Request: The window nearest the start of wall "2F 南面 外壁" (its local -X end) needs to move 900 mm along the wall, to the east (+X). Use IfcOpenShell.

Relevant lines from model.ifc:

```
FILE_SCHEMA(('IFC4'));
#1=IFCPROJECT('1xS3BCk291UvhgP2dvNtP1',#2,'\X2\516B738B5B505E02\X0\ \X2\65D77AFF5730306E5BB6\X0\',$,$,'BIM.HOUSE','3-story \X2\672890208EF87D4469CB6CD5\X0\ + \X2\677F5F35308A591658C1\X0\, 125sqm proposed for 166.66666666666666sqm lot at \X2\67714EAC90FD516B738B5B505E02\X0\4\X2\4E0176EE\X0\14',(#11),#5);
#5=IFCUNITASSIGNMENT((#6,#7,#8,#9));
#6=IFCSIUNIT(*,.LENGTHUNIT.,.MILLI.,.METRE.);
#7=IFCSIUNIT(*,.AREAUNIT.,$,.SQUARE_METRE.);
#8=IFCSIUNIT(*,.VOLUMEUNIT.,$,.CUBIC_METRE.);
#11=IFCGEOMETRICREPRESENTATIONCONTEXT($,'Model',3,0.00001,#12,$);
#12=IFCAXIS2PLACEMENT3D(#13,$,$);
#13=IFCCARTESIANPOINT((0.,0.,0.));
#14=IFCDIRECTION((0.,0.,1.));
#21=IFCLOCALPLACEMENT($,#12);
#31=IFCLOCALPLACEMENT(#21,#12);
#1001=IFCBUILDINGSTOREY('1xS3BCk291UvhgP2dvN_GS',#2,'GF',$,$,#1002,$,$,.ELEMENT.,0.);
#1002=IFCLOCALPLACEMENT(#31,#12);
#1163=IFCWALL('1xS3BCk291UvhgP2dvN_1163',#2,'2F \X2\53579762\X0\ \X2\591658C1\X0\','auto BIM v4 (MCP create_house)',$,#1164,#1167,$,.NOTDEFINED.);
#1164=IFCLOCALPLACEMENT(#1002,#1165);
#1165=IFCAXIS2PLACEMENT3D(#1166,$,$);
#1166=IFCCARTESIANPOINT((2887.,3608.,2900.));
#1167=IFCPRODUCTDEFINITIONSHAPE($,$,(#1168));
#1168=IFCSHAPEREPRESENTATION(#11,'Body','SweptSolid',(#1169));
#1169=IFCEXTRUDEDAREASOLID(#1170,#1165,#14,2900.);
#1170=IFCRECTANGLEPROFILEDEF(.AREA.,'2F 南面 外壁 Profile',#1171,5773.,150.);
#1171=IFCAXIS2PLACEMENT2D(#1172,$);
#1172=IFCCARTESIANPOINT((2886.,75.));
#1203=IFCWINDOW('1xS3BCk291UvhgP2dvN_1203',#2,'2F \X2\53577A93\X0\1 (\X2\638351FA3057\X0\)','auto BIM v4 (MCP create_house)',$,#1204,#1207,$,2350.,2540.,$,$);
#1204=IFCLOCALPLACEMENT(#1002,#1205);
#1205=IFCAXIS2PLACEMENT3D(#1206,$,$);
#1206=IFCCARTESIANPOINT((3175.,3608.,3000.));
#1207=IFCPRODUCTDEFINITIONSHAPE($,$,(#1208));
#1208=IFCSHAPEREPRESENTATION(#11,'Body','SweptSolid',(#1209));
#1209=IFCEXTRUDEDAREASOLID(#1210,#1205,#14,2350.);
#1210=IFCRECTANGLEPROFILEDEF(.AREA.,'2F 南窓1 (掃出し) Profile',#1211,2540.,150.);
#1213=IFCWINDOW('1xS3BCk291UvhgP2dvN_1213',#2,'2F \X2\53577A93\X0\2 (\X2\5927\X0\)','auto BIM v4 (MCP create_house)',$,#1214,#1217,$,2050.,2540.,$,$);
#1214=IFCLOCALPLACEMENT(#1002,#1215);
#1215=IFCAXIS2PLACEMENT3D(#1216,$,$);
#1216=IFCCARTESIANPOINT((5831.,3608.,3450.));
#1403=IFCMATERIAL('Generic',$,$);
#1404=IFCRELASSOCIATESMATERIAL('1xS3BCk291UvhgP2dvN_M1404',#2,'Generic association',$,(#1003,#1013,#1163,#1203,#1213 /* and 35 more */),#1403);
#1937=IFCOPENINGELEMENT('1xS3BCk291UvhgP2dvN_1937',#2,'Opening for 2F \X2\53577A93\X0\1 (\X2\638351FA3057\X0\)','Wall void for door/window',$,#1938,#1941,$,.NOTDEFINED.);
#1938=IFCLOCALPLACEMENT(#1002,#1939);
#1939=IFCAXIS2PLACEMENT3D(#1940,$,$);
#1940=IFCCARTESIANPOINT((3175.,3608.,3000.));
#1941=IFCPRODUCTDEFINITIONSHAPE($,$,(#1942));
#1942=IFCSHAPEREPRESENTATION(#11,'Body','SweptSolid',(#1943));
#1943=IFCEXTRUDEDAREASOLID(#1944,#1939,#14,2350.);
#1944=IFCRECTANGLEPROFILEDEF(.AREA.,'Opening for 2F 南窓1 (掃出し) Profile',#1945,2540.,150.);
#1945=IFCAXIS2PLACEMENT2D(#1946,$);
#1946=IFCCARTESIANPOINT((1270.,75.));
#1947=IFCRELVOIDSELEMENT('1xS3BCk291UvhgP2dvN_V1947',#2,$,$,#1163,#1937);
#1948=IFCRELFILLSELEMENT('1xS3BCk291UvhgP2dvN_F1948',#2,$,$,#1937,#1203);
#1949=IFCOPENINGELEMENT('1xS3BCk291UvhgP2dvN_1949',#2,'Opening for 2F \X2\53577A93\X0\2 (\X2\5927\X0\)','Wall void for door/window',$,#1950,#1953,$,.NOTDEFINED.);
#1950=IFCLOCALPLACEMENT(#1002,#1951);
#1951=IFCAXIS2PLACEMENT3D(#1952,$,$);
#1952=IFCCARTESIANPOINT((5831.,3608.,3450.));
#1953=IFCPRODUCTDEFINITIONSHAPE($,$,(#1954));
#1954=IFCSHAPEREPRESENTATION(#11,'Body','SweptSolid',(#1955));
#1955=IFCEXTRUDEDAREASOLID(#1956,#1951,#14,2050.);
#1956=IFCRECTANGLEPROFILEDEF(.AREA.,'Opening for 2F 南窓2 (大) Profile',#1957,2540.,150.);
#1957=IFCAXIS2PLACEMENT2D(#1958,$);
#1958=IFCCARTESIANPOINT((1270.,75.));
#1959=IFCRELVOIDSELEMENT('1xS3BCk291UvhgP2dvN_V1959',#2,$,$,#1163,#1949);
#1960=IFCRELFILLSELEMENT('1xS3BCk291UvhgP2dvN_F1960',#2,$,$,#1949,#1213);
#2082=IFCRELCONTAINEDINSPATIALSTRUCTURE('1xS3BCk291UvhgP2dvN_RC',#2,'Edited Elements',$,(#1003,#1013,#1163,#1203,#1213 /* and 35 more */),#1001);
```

```python
import ifcopenshell
import ifcopenshell.api.geometry
import ifcopenshell.util.placement

model = ifcopenshell.open("model.ifc")

window = model.by_guid("1xS3BCk291UvhgP2dvN_1203")
opening = window.FillsVoids[0].RelatingOpeningElement
wall = opening.VoidsElements[0].RelatingBuildingElement

wall_matrix = ifcopenshell.util.placement.get_local_placement(wall.ObjectPlacement)
shift = wall_matrix[:3, 0] * 900.0
before = ifcopenshell.util.placement.get_local_placement(window.ObjectPlacement)[:3, 3].copy()

# The window is not placed relative to its opening, so move both.
for product in (opening, window):
    matrix = ifcopenshell.util.placement.get_local_placement(product.ObjectPlacement)
    matrix[:3, 3] += shift
    ifcopenshell.api.geometry.edit_object_placement(model, product=product, matrix=matrix, is_si=False)

after = ifcopenshell.util.placement.get_local_placement(window.ObjectPlacement)[:3, 3]
print("window moved by", (after - before).round(3) + 0.0)

model.write("model-out.ifc")
```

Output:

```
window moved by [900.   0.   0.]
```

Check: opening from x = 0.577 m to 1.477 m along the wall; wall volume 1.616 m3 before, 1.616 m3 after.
